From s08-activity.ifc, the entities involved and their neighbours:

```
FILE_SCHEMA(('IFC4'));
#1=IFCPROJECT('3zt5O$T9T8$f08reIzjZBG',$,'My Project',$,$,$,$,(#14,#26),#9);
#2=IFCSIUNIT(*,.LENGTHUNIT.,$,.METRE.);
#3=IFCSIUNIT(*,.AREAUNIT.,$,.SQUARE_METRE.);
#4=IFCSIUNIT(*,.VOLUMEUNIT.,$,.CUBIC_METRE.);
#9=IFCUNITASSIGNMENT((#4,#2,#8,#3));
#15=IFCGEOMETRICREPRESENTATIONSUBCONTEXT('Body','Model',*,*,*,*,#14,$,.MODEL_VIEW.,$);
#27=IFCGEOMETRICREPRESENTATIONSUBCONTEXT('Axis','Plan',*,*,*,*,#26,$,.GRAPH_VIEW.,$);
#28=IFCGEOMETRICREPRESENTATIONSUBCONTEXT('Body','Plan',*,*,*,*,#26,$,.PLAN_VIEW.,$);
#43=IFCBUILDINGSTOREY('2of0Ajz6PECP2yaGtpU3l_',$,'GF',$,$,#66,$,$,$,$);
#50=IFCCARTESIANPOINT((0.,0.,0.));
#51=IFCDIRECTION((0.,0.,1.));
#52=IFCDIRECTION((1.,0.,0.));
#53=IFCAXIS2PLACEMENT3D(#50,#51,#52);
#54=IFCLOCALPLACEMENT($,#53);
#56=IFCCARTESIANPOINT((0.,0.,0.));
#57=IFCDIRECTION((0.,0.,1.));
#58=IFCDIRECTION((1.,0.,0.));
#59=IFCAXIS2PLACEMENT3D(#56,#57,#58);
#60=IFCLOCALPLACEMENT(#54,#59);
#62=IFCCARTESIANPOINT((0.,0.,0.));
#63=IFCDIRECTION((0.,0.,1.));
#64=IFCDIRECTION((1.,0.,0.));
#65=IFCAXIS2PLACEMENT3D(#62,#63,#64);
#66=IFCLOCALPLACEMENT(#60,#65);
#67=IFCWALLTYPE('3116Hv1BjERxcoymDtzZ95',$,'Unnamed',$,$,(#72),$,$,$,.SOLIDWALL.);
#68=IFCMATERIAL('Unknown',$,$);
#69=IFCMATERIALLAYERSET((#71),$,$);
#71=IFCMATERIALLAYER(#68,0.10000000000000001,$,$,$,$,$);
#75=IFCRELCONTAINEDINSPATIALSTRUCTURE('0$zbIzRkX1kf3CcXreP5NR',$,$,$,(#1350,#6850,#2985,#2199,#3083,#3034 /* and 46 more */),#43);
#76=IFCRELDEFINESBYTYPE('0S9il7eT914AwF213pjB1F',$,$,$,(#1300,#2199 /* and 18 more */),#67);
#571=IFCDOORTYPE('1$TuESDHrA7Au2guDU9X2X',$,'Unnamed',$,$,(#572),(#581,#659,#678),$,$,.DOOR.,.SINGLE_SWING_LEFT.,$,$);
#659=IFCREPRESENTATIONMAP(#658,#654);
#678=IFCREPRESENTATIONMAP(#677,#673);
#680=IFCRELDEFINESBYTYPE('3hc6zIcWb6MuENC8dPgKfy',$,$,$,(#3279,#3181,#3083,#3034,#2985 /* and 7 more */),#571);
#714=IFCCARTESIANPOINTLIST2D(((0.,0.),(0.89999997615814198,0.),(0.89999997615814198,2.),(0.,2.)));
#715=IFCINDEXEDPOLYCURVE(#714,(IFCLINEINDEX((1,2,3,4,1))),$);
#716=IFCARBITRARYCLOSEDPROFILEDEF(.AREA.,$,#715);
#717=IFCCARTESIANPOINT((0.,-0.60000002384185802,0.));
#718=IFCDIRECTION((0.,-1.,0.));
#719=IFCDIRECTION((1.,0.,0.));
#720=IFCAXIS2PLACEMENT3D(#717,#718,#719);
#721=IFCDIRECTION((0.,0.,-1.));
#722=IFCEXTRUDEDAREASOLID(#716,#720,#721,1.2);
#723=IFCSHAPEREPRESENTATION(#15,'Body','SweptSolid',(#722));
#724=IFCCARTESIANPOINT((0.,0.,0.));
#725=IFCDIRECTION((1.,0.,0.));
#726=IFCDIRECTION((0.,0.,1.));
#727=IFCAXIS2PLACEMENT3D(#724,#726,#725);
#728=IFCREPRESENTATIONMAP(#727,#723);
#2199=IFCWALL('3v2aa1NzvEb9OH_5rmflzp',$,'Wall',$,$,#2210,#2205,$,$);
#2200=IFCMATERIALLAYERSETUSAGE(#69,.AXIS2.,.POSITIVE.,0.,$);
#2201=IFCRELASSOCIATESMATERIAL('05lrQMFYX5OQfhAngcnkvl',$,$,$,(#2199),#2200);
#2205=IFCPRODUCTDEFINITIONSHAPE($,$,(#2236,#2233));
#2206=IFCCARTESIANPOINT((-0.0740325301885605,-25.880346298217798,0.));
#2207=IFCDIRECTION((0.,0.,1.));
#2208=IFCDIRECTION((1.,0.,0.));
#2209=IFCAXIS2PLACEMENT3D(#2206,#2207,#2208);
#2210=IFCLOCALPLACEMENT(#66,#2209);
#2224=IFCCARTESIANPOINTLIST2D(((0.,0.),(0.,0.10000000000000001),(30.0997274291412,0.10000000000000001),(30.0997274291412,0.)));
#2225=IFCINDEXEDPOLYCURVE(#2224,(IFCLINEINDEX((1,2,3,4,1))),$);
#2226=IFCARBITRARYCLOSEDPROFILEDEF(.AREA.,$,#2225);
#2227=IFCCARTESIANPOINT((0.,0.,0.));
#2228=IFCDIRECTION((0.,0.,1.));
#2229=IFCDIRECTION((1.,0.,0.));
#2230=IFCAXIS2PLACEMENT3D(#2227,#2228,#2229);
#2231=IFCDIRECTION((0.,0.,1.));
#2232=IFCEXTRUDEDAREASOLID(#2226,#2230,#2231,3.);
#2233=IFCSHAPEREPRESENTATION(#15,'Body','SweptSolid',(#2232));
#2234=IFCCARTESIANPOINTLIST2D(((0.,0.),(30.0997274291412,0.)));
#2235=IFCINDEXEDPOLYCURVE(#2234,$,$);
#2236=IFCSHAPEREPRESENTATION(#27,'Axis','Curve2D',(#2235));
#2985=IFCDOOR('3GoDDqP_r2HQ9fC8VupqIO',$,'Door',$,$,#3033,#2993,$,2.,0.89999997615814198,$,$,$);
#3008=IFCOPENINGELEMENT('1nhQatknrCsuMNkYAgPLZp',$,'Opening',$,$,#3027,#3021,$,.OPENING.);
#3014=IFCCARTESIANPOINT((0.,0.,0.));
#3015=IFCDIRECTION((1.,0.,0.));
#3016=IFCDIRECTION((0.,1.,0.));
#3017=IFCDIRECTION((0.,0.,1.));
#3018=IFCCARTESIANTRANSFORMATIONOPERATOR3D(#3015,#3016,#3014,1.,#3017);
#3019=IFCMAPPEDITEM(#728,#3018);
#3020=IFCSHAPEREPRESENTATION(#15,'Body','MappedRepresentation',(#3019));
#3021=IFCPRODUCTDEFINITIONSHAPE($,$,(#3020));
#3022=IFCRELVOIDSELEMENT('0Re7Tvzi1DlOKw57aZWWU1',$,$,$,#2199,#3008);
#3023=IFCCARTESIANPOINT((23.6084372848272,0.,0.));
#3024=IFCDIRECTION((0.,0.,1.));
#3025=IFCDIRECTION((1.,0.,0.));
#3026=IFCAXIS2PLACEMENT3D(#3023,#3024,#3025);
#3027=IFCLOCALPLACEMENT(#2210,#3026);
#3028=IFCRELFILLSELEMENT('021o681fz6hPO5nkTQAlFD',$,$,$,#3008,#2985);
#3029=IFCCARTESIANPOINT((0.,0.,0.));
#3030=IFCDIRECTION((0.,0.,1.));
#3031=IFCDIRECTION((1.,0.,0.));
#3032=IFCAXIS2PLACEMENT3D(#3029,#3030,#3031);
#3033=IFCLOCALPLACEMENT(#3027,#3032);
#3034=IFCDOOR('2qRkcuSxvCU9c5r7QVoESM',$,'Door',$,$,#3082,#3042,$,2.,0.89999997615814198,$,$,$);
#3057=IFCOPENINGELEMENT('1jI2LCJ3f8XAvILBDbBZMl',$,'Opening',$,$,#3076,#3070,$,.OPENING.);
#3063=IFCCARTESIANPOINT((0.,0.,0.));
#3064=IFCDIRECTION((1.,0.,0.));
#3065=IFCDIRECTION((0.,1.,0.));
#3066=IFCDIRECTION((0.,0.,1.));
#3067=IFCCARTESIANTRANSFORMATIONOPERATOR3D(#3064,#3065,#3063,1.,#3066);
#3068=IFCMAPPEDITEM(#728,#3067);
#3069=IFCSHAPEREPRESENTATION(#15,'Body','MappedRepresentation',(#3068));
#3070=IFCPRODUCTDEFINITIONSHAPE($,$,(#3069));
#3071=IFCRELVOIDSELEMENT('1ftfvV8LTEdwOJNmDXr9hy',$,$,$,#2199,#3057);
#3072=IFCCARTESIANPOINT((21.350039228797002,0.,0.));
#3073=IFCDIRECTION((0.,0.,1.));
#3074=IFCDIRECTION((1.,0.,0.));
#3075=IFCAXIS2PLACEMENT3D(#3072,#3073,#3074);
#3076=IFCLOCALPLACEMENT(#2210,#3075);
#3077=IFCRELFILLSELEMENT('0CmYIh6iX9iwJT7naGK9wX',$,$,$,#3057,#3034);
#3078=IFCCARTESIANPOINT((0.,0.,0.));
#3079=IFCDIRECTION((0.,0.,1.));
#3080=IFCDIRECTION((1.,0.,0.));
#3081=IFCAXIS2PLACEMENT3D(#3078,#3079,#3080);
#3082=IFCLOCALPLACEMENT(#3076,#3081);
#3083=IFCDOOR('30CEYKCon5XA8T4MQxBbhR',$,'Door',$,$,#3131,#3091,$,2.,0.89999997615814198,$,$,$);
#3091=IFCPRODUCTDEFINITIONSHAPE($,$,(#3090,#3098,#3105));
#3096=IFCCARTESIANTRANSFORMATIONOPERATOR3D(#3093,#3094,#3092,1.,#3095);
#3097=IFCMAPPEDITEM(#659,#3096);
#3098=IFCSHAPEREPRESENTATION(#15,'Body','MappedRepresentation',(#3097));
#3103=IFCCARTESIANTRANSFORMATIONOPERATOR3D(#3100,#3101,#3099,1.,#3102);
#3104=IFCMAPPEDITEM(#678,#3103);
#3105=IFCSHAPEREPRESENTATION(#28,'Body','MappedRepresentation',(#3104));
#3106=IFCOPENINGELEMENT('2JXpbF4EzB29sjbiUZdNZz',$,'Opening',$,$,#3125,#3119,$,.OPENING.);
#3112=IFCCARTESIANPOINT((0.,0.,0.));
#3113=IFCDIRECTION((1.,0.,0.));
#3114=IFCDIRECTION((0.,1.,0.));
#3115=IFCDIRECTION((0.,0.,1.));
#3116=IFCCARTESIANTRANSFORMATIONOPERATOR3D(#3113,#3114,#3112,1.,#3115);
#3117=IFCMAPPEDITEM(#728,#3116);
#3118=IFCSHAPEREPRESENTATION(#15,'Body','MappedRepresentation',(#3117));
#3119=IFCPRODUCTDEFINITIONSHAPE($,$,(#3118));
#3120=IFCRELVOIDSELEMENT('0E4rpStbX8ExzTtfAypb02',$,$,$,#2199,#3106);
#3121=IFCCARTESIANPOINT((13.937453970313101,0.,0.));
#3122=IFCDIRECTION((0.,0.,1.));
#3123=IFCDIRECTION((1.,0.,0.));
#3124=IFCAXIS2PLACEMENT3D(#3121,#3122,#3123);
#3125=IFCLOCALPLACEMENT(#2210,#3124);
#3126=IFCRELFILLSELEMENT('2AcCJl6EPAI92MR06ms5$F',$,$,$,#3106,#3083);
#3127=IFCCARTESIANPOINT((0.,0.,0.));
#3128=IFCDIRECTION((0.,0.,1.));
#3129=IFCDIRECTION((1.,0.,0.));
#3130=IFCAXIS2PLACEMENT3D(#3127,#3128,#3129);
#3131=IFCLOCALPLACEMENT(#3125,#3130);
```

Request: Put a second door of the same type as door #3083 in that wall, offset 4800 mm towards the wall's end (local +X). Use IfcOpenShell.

```python
import ifcopenshell
import ifcopenshell.api.feature
import ifcopenshell.api.geometry
import ifcopenshell.api.root
import ifcopenshell.geom
import ifcopenshell.util.element
import ifcopenshell.util.placement
import ifcopenshell.util.shape

model = ifcopenshell.open("s08-activity.ifc")
settings = ifcopenshell.geom.settings()


def volume(element):
    """Net volume in cubic metres, openings subtracted."""
    shape = ifcopenshell.geom.create_shape(settings, element)
    return ifcopenshell.util.shape.get_volume(shape.geometry)


door = model.by_id(3083)
opening = door.FillsVoids[0].RelatingOpeningElement
wall = opening.VoidsElements[0].RelatingBuildingElement
before = volume(wall)
shift = ifcopenshell.util.placement.get_local_placement(wall.ObjectPlacement)[:3, 0] * 4.8

# copy_class copies the void relationship, type, container and properties, but no geometry.
new_opening = ifcopenshell.api.root.copy_class(model, product=opening)
new_opening.Representation = ifcopenshell.util.element.copy_deep(
    model, opening.Representation, exclude=["IfcGeometricRepresentationContext", "IfcRepresentationMap"]
)
new_door = ifcopenshell.api.root.copy_class(model, product=door)
new_door.Representation = ifcopenshell.util.element.copy_deep(
    model, door.Representation, exclude=["IfcGeometricRepresentationContext", "IfcRepresentationMap"]
)
ifcopenshell.api.feature.add_filling(model, opening=new_opening, element=new_door)

for old, new in ((opening, new_opening), (door, new_door)):
    matrix = ifcopenshell.util.placement.get_local_placement(old.ObjectPlacement)
    matrix[:3, 3] += shift
    ifcopenshell.api.geometry.edit_object_placement(model, product=new, matrix=matrix, is_si=False)

after = volume(wall)

print(f"wall volume {before:.3f} -> {after:.3f} m3")

model.write("s08-activity_edited.ifc")
```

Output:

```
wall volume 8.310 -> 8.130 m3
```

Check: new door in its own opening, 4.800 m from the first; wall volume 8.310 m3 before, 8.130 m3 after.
